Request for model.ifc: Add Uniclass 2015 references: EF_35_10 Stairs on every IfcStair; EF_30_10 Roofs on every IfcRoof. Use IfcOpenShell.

First a look at what the model holds.

```python
import ifcopenshell

model = ifcopenshell.open("model.ifc")
print(model.schema)
print("classifications:", [c.Name for c in model.by_type("IfcClassification")])
for ifc_class in ("IfcDoor", "IfcRoof", "IfcStair", "IfcWall", "IfcWindow"):
    print(ifc_class, len(model.by_type(ifc_class)))
```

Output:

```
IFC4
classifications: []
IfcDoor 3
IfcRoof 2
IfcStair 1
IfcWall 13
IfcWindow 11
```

```python
import ifcopenshell
import ifcopenshell.api.classification

model = ifcopenshell.open("model.ifc")

system = ifcopenshell.api.classification.add_classification(model, classification="Uniclass 2015")

codes = {
    "IfcStair": ("EF_35_10", "Stairs"),
    "IfcRoof": ("EF_30_10", "Roofs"),
}
for ifc_class, (code, name) in codes.items():
    products = model.by_type(ifc_class)
    ifcopenshell.api.classification.add_reference(
        model, products=products, classification=system, identification=code, name=name
    )
    print(code, len(products))

model.write("model_rev.ifc")
```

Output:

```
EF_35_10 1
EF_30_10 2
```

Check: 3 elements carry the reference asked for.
